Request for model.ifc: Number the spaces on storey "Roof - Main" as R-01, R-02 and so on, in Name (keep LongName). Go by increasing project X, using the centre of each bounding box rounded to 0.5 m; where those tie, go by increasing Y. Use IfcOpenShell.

First a look at what the model holds.

```python
import ifcopenshell
import ifcopenshell.util.element
import ifcopenshell.util.placement

model = ifcopenshell.open("model.ifc")
print(model.schema)
storey = next(s for s in model.by_type("IfcBuildingStorey") if s.Name == "Roof - Main")
spaces = [e for e in ifcopenshell.util.element.get_decomposition(storey) if e.is_a("IfcSpace")]
for e in sorted(spaces, key=lambda e: e.id()):
    origin = ifcopenshell.util.placement.get_local_placement(e.ObjectPlacement)[:3, 3]
    print(e.id(), e.Name, e.LongName, origin.round(2) + 0.0, sep=" | ")
```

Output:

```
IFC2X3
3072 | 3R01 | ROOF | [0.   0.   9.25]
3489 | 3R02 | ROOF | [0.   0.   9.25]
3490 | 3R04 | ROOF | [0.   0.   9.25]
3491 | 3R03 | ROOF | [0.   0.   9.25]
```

```python
import ifcopenshell
import ifcopenshell.geom
import ifcopenshell.util.element
import ifcopenshell.util.shape

model = ifcopenshell.open("model.ifc")
settings = ifcopenshell.geom.settings()
settings.set("use-world-coords", True)


def centre(element):
    shape = ifcopenshell.geom.create_shape(settings, element)
    return ifcopenshell.util.shape.get_bbox_centroid(shape.geometry)


storey = next(s for s in model.by_type("IfcBuildingStorey") if s.Name == "Roof - Main")
spaces = [e for e in ifcopenshell.util.element.get_decomposition(storey) if e.is_a("IfcSpace")]

# Insertion points can sit at a corner or the storey origin, so sort by the geometry (in metres).
centres = {e: centre(e) for e in spaces}
spaces.sort(key=lambda e: (round(centres[e][0] / 0.5), centres[e][1]))

for i, e in enumerate(spaces, start=1):
    number = f"R-{i:02d}"
    e.Name = number
    print(e.id(), number)

model.write("model_edited.ifc")
```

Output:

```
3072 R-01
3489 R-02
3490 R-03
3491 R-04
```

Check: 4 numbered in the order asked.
